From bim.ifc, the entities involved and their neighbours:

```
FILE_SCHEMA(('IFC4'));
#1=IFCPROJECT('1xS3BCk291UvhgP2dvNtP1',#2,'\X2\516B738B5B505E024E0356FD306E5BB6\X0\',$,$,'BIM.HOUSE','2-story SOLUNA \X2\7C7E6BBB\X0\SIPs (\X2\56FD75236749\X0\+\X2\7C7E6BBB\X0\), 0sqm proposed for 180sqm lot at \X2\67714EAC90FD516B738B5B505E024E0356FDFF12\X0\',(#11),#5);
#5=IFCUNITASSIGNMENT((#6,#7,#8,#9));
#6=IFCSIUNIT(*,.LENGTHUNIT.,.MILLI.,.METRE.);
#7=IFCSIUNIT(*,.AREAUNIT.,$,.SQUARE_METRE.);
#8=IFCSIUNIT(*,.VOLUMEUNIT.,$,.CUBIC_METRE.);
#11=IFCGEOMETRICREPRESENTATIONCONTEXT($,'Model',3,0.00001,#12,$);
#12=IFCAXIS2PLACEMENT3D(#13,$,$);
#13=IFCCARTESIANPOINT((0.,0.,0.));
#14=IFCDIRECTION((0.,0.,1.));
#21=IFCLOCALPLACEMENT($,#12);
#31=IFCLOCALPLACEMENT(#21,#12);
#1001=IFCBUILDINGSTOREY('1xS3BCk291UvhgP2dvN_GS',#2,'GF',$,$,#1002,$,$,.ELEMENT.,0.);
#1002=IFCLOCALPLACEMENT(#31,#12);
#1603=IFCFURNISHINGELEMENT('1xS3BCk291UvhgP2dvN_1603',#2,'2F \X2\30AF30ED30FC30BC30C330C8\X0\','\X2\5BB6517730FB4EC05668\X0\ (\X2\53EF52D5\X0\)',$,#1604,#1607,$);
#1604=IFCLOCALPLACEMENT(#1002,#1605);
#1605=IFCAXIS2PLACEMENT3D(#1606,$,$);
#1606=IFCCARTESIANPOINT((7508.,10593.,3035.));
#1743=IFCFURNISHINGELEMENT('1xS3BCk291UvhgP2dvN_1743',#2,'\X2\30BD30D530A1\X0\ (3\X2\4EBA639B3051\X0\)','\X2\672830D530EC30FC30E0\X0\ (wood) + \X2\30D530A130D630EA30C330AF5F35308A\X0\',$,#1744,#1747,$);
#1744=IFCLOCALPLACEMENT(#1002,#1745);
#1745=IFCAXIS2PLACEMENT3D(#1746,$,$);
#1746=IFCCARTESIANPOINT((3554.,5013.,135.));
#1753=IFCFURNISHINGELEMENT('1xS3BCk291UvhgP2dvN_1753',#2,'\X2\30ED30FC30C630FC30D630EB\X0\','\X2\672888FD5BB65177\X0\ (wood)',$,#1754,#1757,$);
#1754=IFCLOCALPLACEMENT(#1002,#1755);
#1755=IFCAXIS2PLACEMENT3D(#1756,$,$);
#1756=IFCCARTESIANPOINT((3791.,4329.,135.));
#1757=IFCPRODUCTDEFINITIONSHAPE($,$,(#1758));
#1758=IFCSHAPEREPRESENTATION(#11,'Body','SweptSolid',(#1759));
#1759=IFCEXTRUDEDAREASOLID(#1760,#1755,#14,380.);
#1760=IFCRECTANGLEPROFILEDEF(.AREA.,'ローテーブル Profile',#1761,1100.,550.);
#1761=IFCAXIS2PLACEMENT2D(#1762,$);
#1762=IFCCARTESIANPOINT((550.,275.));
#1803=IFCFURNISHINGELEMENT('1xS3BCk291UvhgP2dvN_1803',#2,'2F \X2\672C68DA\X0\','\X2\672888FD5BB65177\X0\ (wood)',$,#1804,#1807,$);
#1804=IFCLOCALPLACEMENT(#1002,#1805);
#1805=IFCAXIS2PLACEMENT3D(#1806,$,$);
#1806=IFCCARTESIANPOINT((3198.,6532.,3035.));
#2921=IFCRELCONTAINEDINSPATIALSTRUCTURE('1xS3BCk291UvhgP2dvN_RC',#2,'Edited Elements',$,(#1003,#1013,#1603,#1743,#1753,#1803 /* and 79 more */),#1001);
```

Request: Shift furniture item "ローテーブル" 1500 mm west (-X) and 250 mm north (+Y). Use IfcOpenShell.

```python
import ifcopenshell
import ifcopenshell.api.geometry
import ifcopenshell.util.placement

model = ifcopenshell.open("bim.ifc")

item = model.by_guid("1xS3BCk291UvhgP2dvN_1753")
matrix = ifcopenshell.util.placement.get_local_placement(item.ObjectPlacement)
matrix[0, 3] -= 1500.0
matrix[1, 3] += 250.0
ifcopenshell.api.geometry.edit_object_placement(model, product=item, matrix=matrix, is_si=False)

print(ifcopenshell.util.placement.get_local_placement(item.ObjectPlacement).round(3) + 0.0)

model.write("bim_edited.ifc")
```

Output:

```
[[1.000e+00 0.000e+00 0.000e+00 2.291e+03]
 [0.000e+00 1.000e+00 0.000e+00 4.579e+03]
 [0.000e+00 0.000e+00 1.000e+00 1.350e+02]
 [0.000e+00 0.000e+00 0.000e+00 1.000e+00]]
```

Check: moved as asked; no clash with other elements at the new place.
